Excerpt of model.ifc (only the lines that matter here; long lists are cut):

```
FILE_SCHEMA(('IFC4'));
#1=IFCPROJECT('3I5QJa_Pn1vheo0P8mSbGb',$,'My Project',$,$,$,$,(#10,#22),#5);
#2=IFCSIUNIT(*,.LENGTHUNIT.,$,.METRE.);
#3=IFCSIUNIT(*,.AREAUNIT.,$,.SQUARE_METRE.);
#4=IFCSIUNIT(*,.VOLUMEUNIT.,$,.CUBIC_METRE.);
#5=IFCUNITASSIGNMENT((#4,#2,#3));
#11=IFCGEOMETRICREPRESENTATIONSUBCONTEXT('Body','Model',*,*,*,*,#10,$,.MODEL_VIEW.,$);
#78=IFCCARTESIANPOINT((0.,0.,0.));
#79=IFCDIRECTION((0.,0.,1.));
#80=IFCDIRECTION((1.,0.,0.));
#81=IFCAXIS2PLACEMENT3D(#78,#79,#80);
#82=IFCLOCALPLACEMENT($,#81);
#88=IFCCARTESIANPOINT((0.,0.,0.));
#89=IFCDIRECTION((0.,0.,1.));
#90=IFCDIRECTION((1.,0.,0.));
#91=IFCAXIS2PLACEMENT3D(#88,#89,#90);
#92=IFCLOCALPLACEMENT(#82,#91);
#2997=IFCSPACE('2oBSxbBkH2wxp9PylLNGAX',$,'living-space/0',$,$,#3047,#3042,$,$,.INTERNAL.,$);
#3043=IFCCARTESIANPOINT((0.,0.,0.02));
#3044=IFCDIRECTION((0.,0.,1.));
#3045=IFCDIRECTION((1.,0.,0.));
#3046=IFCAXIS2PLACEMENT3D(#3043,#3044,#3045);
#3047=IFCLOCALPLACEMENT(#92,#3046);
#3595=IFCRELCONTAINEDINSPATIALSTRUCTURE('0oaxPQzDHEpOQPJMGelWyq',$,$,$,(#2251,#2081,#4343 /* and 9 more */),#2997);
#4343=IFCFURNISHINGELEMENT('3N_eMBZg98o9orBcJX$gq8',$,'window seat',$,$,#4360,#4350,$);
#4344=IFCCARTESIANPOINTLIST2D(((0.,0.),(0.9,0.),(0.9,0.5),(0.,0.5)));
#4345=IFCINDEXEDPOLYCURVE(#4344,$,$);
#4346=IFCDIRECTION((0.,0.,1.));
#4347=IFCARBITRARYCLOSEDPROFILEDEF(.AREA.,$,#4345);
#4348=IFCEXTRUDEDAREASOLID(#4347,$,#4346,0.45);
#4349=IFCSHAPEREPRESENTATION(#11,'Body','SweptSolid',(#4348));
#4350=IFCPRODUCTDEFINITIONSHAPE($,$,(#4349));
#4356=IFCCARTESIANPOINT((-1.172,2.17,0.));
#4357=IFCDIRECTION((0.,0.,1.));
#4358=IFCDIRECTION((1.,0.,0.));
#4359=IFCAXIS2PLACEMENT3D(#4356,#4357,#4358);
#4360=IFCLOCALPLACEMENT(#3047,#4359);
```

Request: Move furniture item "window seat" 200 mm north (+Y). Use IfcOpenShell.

```python
import ifcopenshell
import ifcopenshell.api.geometry
import ifcopenshell.util.placement
import ifcopenshell.util.unit

model = ifcopenshell.open("model.ifc")
unit_scale = ifcopenshell.util.unit.calculate_unit_scale(model)

item = model.by_guid("3N_eMBZg98o9orBcJX$gq8")
matrix = ifcopenshell.util.placement.get_local_placement(item.ObjectPlacement)
matrix[1, 3] += 0.2 / unit_scale
ifcopenshell.api.geometry.edit_object_placement(model, product=item, matrix=matrix, is_si=False)

print(ifcopenshell.util.placement.get_local_placement(item.ObjectPlacement).round(3) + 0.0)

model.write("model-out.ifc")
```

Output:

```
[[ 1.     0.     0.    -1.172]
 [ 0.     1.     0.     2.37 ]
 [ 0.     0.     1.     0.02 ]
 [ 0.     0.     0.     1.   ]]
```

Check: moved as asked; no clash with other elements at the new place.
